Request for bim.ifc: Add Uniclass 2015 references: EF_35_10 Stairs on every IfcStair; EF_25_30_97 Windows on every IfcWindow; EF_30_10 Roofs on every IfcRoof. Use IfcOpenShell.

First a look at what the model holds.

```python
import ifcopenshell

model = ifcopenshell.open("bim.ifc")
print(model.schema)
print("classifications:", [c.Name for c in model.by_type("IfcClassification")])
for ifc_class in ("IfcDoor", "IfcRoof", "IfcStair", "IfcWall", "IfcWindow"):
    print(ifc_class, len(model.by_type(ifc_class)))
```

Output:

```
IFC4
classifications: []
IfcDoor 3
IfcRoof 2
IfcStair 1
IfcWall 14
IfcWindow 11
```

```python
import ifcopenshell
import ifcopenshell.api.classification

model = ifcopenshell.open("bim.ifc")

system = ifcopenshell.api.classification.add_classification(model, classification="Uniclass 2015")

codes = {
    "IfcStair": ("EF_35_10", "Stairs"),
    "IfcWindow": ("EF_25_30_97", "Windows"),
    "IfcRoof": ("EF_30_10", "Roofs"),
}
for ifc_class, (code, name) in codes.items():
    products = model.by_type(ifc_class)
    ifcopenshell.api.classification.add_reference(
        model, products=products, classification=system, identification=code, name=name
    )
    print(code, len(products))

model.write("bim_edited.ifc")
```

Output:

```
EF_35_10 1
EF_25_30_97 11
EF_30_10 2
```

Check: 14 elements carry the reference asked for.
